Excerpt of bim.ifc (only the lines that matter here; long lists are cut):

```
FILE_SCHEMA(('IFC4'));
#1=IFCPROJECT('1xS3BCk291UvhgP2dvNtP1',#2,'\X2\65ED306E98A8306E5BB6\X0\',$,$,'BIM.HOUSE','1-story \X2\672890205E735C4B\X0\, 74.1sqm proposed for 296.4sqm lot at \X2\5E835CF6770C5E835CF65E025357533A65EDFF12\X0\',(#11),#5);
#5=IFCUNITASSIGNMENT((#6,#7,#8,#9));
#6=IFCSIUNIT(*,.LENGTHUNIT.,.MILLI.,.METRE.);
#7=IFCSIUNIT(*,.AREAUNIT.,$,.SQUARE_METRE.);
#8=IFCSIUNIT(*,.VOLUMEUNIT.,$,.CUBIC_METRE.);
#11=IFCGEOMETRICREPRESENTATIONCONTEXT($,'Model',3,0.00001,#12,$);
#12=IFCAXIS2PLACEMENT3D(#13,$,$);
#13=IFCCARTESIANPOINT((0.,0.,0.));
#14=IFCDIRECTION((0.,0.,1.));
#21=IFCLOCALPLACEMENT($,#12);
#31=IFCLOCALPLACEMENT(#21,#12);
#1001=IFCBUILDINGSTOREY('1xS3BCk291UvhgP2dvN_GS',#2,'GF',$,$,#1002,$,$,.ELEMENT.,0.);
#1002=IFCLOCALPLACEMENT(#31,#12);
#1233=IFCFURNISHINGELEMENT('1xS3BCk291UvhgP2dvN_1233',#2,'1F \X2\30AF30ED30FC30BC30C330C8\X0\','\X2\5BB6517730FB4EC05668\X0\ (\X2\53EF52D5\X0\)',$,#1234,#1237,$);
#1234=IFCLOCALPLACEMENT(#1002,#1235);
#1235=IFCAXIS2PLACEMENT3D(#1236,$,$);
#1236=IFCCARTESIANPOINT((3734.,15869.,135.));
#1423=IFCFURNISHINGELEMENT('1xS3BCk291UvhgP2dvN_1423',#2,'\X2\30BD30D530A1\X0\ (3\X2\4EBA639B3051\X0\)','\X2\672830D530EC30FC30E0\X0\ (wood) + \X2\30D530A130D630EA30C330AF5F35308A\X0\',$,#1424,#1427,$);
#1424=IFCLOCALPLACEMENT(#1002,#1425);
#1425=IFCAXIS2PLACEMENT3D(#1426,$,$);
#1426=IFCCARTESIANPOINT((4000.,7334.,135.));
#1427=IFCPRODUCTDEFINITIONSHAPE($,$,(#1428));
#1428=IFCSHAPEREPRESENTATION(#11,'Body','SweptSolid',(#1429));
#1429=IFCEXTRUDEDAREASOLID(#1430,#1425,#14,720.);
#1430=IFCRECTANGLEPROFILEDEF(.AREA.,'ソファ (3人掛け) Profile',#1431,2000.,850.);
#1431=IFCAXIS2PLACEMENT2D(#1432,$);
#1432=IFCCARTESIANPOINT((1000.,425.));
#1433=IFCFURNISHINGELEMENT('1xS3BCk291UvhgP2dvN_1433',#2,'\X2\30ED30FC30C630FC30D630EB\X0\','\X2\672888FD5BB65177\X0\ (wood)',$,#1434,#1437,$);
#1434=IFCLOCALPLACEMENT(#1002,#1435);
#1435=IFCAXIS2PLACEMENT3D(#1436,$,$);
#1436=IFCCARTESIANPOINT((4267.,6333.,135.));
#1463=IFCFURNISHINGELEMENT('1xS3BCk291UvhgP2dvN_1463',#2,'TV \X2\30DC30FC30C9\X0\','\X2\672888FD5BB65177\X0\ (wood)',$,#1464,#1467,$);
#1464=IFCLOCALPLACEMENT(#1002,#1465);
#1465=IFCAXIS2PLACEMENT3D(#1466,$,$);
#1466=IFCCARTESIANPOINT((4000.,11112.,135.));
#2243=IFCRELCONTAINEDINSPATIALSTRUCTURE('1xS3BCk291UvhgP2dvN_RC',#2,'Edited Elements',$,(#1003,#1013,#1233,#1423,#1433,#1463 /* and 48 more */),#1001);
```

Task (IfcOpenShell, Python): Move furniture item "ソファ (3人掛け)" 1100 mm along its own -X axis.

```python
import ifcopenshell
import ifcopenshell.api.geometry
import ifcopenshell.util.placement

model = ifcopenshell.open("bim.ifc")

item = model.by_guid("1xS3BCk291UvhgP2dvN_1423")
matrix = ifcopenshell.util.placement.get_local_placement(item.ObjectPlacement)
matrix[:3, 3] -= matrix[:3, 0] * 1100.0
ifcopenshell.api.geometry.edit_object_placement(model, product=item, matrix=matrix, is_si=False)

print(ifcopenshell.util.placement.get_local_placement(item.ObjectPlacement).round(3) + 0.0)

model.write("bim_edited.ifc")
```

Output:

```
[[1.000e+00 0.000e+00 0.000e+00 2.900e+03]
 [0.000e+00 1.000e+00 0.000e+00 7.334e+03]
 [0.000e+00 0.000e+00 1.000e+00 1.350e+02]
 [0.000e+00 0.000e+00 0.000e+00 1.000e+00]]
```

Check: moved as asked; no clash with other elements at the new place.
